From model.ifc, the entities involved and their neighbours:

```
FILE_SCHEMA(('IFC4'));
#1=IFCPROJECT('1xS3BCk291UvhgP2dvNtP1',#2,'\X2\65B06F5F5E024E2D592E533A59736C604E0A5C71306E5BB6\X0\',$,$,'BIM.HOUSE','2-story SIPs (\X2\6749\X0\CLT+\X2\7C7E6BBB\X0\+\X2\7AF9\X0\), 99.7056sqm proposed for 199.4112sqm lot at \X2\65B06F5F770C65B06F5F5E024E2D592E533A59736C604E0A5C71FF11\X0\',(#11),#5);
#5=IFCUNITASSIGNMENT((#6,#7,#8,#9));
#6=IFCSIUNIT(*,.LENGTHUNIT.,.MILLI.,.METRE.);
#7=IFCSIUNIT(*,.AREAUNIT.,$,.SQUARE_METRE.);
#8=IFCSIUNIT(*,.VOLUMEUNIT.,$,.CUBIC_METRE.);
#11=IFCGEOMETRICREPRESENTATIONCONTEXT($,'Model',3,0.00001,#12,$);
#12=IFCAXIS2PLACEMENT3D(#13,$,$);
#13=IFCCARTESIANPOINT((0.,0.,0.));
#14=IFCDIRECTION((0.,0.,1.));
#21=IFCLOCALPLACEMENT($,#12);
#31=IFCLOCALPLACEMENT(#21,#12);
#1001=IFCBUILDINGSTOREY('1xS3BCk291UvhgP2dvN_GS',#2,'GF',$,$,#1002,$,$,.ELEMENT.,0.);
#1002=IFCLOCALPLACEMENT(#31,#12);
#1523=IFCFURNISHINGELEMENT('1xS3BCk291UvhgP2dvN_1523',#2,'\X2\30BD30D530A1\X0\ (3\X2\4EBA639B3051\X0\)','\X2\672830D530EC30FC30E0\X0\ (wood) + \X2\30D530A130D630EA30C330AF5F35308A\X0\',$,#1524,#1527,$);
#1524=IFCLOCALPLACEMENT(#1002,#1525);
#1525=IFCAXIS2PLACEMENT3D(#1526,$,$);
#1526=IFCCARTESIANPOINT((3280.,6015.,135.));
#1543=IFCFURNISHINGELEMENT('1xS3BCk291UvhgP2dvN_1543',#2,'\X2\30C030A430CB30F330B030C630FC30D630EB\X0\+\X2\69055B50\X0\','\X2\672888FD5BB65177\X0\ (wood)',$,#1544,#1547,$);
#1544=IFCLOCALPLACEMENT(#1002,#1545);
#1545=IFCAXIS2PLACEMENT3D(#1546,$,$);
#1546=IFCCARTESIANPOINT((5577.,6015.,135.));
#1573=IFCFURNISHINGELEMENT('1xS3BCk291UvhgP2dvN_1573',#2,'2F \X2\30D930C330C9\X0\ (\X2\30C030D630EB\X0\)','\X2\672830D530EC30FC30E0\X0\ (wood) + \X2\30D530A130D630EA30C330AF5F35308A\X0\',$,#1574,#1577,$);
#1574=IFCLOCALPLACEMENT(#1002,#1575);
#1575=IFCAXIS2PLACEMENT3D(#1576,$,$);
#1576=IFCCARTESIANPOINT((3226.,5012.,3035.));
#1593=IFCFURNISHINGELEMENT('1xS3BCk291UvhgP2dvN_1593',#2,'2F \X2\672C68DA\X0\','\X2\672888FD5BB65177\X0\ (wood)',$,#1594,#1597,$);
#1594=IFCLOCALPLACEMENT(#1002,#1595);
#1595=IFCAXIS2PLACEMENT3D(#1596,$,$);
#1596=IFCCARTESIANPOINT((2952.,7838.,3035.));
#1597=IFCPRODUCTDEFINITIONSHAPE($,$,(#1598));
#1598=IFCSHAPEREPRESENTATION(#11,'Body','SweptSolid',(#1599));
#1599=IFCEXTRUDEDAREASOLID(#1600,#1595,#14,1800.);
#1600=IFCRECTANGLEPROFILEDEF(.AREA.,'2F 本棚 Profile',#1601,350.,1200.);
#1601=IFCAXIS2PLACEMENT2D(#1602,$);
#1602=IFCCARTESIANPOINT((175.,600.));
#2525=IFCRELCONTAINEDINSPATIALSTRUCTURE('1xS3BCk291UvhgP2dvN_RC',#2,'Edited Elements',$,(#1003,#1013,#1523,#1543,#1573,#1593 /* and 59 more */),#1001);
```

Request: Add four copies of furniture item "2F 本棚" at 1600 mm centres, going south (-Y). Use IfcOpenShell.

```python
import numpy as np
import ifcopenshell
import ifcopenshell.api.geometry
import ifcopenshell.api.root
import ifcopenshell.util.element
import ifcopenshell.util.placement

model = ifcopenshell.open("model.ifc")


def reuse_history(source, copy):
    """copy_class also copies each property set's owner history, people and application; keep the originals."""
    for rel in copy.IsDefinedBy:
        if rel.is_a("IfcRelDefinesByProperties") and (history := rel.RelatingPropertyDefinition.OwnerHistory):
            rel.RelatingPropertyDefinition.OwnerHistory = source.OwnerHistory
            ifcopenshell.util.element.remove_deep2(model, history)


source = model.by_guid("1xS3BCk291UvhgP2dvN_1593")
base = ifcopenshell.util.placement.get_local_placement(source.ObjectPlacement)
step = np.array([0.0, -1.0, 0.0]) * 1600.0

for i in range(1, 5):
    copy = ifcopenshell.api.root.copy_class(model, product=source)
    copy.Representation = ifcopenshell.util.element.copy_deep(
        model, source.Representation, exclude=["IfcGeometricRepresentationContext", "IfcRepresentationMap"]
    )
    reuse_history(source, copy)
    matrix = base.copy()
    matrix[:3, 3] += i * step
    print("added at", matrix[:3, 3].round(3) + 0.0)
    ifcopenshell.api.geometry.edit_object_placement(model, product=copy, matrix=matrix, is_si=False)

model.write("model_rev.ifc")
```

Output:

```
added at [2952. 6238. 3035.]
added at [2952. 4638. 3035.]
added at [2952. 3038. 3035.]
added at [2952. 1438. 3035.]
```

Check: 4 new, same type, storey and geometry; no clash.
